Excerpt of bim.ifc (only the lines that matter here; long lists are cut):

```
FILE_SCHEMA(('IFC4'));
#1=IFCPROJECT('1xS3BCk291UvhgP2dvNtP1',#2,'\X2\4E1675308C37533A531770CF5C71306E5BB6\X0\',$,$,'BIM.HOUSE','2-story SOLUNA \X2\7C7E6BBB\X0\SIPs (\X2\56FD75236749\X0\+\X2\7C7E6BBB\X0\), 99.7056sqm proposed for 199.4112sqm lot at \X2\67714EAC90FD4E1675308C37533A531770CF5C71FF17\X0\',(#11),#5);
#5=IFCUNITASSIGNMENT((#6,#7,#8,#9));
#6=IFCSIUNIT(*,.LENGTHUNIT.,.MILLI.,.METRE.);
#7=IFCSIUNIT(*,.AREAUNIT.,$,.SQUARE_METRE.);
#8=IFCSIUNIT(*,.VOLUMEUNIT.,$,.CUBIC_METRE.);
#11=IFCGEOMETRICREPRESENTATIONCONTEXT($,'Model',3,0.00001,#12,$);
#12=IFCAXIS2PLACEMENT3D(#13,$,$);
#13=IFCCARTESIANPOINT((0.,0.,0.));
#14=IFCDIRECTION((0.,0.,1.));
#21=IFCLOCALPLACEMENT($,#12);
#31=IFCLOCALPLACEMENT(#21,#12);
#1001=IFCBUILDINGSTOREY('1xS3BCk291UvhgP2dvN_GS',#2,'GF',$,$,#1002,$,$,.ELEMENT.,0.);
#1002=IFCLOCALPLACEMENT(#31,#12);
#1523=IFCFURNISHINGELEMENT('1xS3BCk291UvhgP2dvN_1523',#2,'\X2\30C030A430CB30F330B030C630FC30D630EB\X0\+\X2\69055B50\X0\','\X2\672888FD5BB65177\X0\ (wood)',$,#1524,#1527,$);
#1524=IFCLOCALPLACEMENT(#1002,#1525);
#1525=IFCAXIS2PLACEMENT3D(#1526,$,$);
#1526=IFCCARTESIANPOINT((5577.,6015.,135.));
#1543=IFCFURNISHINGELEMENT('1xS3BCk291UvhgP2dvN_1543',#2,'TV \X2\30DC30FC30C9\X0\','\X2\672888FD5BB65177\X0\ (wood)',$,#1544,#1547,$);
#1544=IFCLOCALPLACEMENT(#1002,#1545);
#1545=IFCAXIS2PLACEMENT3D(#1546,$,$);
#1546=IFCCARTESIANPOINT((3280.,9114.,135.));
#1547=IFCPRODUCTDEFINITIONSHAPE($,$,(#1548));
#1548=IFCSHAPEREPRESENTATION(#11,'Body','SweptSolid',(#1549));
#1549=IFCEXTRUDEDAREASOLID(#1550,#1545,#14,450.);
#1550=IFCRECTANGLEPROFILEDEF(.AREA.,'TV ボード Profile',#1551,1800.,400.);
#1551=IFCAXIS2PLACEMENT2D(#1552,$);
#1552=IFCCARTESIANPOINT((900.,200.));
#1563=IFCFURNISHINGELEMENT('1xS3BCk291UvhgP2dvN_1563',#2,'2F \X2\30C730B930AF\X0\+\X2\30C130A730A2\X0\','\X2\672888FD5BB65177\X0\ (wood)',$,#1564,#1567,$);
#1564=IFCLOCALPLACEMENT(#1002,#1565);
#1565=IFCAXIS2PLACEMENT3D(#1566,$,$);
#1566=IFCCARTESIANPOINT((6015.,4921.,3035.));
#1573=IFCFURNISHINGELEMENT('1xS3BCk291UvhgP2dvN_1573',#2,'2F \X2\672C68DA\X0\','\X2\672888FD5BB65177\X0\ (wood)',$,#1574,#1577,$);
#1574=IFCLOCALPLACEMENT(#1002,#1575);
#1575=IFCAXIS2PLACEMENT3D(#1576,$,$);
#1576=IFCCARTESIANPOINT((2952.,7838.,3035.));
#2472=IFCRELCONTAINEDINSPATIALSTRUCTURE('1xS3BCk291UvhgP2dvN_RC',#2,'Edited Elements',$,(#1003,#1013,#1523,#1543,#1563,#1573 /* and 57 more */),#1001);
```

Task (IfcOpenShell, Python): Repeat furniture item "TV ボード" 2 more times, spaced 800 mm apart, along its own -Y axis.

```python
import ifcopenshell
import ifcopenshell.api.geometry
import ifcopenshell.api.root
import ifcopenshell.util.element
import ifcopenshell.util.placement
import ifcopenshell.util.unit

model = ifcopenshell.open("bim.ifc")
unit_scale = ifcopenshell.util.unit.calculate_unit_scale(model)


def reuse_history(source, copy):
    """copy_class also copies each property set's owner history, people and application; keep the originals."""
    for rel in copy.IsDefinedBy:
        if rel.is_a("IfcRelDefinesByProperties") and (history := rel.RelatingPropertyDefinition.OwnerHistory):
            rel.RelatingPropertyDefinition.OwnerHistory = source.OwnerHistory
            ifcopenshell.util.element.remove_deep2(model, history)


source = model.by_id(1543)
base = ifcopenshell.util.placement.get_local_placement(source.ObjectPlacement)
step = -base[:3, 1] * 0.8 / unit_scale

for i in range(1, 3):
    copy = ifcopenshell.api.root.copy_class(model, product=source)
    copy.Representation = ifcopenshell.util.element.copy_deep(
        model, source.Representation, exclude=["IfcGeometricRepresentationContext", "IfcRepresentationMap"]
    )
    reuse_history(source, copy)
    matrix = base.copy()
    matrix[:3, 3] += i * step
    print("added at", matrix[:3, 3].round(3) + 0.0)
    ifcopenshell.api.geometry.edit_object_placement(model, product=copy, matrix=matrix, is_si=False)

model.write("bim_v2.ifc")
```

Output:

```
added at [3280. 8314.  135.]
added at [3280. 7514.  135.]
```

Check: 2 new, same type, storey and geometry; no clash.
